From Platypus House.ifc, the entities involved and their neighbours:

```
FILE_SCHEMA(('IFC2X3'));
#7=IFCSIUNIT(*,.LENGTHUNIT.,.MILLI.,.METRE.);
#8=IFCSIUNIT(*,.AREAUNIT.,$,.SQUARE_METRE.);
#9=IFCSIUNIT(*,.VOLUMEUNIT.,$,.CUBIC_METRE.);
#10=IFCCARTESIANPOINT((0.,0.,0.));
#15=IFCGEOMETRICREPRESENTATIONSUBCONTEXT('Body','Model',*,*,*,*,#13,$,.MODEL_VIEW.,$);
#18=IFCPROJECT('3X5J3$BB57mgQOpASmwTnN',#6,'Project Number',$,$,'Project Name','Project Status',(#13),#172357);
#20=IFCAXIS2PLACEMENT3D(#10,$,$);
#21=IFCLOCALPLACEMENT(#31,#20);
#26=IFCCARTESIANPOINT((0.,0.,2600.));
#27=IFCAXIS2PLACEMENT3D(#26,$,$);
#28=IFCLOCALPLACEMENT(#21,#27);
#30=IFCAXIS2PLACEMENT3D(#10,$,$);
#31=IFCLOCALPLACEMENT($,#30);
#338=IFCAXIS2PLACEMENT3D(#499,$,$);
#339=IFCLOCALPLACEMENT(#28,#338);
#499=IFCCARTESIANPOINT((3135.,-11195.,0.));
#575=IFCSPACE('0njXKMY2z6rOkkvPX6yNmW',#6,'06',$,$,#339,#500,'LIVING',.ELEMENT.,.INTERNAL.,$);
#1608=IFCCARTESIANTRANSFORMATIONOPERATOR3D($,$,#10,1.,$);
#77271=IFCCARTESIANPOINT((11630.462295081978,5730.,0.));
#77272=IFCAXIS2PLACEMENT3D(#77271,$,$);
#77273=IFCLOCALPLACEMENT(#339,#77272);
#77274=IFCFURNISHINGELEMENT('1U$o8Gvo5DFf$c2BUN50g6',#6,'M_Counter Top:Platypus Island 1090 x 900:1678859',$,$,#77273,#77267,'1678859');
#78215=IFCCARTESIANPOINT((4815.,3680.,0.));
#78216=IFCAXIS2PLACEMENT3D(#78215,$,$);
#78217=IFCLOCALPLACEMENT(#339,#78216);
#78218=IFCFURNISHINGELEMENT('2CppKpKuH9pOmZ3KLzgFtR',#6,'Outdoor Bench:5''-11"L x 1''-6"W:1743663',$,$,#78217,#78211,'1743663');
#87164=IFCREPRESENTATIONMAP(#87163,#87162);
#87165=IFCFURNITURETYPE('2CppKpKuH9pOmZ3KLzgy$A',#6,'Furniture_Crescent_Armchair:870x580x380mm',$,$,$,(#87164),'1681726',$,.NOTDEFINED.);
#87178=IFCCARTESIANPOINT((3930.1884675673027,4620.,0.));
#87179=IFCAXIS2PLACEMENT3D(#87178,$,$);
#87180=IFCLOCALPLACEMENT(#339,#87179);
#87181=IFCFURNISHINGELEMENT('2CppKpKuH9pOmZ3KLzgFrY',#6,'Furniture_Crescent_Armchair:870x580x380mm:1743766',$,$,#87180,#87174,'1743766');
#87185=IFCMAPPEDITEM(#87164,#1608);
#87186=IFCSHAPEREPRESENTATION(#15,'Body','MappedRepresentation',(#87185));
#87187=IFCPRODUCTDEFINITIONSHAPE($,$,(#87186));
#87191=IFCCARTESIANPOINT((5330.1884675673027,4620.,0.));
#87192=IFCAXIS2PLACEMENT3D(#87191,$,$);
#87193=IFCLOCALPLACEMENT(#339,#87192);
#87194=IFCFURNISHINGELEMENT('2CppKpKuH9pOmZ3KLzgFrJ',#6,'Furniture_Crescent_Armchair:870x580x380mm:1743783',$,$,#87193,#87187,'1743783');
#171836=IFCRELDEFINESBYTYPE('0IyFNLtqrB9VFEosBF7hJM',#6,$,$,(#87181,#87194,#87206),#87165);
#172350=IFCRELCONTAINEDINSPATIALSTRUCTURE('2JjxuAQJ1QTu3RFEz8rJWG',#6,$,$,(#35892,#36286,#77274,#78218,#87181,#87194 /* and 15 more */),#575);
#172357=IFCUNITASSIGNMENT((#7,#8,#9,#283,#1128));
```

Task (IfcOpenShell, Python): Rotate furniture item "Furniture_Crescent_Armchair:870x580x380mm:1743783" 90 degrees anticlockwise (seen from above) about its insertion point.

```python
import ifcopenshell
import ifcopenshell.api.geometry
import ifcopenshell.util.placement

model = ifcopenshell.open("Platypus House.ifc")

item = model.by_guid("2CppKpKuH9pOmZ3KLzgFrJ")
matrix = ifcopenshell.util.placement.get_local_placement(item.ObjectPlacement)
matrix = matrix @ ifcopenshell.util.placement.rotation(90, "Z")
ifcopenshell.api.geometry.edit_object_placement(model, product=item, matrix=matrix, is_si=False)

print(ifcopenshell.util.placement.get_local_placement(item.ObjectPlacement).round(3) + 0.0)

model.write("Platypus House-out.ifc")
```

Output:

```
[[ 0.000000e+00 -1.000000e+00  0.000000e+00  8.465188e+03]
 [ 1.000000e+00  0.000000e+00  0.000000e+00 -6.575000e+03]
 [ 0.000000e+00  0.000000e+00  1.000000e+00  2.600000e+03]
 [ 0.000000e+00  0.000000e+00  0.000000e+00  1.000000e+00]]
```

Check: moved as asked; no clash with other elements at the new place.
